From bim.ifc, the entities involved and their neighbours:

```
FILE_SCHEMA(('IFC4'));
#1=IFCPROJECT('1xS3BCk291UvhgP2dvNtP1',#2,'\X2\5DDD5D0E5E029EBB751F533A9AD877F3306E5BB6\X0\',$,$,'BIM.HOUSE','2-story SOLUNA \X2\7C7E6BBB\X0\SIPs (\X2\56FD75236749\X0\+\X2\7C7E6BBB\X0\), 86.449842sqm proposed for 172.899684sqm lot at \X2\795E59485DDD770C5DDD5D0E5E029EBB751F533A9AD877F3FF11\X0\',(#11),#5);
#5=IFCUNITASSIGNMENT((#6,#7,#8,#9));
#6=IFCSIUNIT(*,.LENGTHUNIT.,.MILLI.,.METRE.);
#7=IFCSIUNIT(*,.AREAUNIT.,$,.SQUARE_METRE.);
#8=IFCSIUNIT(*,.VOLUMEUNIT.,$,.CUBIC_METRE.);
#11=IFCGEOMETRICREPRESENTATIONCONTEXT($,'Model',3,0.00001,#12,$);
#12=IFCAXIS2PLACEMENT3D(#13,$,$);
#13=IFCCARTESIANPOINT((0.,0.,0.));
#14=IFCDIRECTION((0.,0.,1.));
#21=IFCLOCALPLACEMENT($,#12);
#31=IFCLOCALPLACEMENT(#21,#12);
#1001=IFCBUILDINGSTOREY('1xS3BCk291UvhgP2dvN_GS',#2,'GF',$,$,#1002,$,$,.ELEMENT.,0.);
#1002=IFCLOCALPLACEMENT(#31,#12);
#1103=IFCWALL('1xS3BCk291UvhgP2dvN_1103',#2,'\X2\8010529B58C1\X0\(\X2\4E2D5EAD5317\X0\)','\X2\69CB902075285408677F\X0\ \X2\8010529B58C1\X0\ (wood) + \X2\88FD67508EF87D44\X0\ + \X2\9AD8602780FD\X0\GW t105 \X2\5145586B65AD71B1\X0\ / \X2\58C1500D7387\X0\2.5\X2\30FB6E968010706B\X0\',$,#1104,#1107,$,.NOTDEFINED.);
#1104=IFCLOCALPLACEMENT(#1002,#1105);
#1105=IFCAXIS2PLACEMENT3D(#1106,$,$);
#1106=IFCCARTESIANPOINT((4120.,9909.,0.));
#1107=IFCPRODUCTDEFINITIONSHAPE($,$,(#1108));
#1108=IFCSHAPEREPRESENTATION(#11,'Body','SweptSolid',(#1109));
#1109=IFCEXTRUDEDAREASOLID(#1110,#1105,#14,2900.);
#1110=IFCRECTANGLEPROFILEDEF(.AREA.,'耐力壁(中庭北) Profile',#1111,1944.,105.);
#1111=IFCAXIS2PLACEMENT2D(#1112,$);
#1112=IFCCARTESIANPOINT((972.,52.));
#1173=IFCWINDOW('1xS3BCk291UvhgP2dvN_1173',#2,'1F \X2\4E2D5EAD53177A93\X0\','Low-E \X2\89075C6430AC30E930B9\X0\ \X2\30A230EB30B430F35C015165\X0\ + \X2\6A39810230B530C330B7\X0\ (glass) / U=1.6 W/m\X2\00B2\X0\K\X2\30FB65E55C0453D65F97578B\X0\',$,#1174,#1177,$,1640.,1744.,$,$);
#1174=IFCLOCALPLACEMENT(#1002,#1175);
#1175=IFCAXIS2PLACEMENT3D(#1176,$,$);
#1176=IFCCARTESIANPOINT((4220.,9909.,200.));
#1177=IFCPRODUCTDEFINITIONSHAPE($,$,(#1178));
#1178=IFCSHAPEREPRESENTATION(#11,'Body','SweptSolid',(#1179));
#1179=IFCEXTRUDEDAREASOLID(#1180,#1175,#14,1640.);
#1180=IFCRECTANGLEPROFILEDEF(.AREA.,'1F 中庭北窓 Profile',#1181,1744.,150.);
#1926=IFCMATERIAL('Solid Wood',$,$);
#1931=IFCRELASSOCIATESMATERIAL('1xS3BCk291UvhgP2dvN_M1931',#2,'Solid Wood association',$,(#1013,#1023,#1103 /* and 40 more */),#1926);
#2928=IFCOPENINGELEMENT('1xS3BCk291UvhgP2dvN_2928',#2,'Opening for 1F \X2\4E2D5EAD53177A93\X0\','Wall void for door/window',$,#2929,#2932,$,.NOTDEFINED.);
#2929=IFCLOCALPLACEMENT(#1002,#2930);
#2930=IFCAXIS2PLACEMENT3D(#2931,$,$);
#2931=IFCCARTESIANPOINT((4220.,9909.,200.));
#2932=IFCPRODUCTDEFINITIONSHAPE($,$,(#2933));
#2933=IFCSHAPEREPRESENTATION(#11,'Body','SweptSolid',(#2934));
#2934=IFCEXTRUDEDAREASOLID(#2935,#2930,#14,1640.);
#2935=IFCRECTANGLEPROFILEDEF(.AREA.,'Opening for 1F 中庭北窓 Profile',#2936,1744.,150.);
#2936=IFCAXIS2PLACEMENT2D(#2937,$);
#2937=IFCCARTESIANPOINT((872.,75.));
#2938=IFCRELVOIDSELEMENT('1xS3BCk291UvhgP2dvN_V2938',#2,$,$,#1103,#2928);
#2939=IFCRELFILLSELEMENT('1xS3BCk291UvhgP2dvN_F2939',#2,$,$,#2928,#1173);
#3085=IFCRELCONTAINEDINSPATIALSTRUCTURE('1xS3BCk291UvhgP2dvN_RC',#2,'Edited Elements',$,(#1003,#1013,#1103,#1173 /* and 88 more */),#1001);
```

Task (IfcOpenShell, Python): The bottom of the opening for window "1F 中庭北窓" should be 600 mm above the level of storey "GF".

```python
import numpy as np
import ifcopenshell
import ifcopenshell.api.geometry
import ifcopenshell.geom
import ifcopenshell.util.element
import ifcopenshell.util.placement
import ifcopenshell.util.shape
import ifcopenshell.util.unit

model = ifcopenshell.open("bim.ifc")
unit_scale = ifcopenshell.util.unit.calculate_unit_scale(model)

window = model.by_guid("1xS3BCk291UvhgP2dvN_1173")
opening = window.FillsVoids[0].RelatingOpeningElement
storey = ifcopenshell.util.element.get_container(window, ifc_class="IfcBuildingStorey")
level = ifcopenshell.util.placement.get_local_placement(storey.ObjectPlacement)[2, 3]

# The opening's origin need not be at the sill, so measure its lowest point.
shape = ifcopenshell.geom.create_shape(ifcopenshell.geom.settings(), opening)
bottom = ifcopenshell.util.shape.get_shape_bottom_elevation(shape, shape.geometry) / unit_scale
dz = level + 0.6 / unit_scale - bottom

shift = np.array([0.0, 0.0, dz])
# The window is not placed relative to its opening, so move both.
for product in (opening, window):
    matrix = ifcopenshell.util.placement.get_local_placement(product.ObjectPlacement)
    matrix[:3, 3] += shift
    ifcopenshell.api.geometry.edit_object_placement(model, product=product, matrix=matrix, is_si=False)

print(f"moved by {dz * unit_scale:+.3f} m")

model.write("bim_v2.ifc")
```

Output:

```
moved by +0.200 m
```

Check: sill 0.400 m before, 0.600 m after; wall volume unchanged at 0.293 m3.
